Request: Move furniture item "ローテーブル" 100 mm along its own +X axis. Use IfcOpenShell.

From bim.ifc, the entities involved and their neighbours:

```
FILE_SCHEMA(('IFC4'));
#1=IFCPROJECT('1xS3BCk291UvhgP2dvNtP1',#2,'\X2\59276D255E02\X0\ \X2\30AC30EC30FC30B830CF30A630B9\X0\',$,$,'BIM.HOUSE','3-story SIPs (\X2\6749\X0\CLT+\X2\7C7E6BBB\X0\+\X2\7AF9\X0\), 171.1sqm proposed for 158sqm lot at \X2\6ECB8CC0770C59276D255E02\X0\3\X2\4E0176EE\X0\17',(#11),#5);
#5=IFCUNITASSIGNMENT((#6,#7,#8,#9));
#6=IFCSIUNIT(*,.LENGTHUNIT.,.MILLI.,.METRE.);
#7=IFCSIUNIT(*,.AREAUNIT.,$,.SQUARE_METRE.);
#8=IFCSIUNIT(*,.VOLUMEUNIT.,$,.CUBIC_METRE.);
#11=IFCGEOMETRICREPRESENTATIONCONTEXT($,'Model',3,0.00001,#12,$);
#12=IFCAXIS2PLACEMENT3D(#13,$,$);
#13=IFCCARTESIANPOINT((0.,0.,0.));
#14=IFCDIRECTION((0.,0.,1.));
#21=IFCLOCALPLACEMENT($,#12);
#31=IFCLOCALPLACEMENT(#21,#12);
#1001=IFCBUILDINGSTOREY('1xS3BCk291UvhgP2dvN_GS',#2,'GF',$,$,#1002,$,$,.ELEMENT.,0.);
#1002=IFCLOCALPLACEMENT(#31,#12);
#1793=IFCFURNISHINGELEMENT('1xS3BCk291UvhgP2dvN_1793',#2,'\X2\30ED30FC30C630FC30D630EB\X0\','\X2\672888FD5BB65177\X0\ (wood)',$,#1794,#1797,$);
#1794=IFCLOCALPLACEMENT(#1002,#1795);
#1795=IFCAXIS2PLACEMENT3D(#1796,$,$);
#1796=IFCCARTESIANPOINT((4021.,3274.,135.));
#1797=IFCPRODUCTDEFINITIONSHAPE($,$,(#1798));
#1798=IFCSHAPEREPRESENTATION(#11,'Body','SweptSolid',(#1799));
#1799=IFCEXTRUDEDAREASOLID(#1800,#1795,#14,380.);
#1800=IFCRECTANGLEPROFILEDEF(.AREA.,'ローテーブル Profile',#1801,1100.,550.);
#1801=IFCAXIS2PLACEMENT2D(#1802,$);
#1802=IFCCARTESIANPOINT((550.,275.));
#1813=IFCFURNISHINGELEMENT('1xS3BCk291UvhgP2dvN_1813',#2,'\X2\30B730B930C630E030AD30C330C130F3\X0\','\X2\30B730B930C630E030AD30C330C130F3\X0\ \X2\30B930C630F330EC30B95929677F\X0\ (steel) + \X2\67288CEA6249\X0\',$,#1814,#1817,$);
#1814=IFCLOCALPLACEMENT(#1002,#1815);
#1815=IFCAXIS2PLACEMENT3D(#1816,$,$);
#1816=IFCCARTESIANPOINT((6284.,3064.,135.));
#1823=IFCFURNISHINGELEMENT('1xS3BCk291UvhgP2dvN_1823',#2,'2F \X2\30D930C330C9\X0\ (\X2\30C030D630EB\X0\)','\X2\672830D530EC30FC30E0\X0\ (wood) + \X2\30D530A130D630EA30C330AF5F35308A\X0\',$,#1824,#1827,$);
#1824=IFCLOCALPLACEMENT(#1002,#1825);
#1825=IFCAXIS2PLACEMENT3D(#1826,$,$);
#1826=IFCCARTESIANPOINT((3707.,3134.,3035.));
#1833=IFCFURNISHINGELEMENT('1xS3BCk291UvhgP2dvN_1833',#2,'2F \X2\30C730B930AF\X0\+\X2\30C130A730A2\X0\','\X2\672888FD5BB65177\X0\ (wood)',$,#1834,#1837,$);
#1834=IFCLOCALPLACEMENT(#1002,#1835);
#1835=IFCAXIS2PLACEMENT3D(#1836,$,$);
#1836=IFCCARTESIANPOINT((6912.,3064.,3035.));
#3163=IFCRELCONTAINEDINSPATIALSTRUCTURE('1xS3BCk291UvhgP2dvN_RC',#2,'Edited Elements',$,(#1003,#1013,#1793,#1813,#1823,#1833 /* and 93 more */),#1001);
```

```python
import ifcopenshell
import ifcopenshell.api.geometry
import ifcopenshell.util.placement
import ifcopenshell.util.unit

model = ifcopenshell.open("bim.ifc")
unit_scale = ifcopenshell.util.unit.calculate_unit_scale(model)

item = model.by_guid("1xS3BCk291UvhgP2dvN_1793")
matrix = ifcopenshell.util.placement.get_local_placement(item.ObjectPlacement)
matrix[:3, 3] += matrix[:3, 0] * 0.1 / unit_scale
ifcopenshell.api.geometry.edit_object_placement(model, product=item, matrix=matrix, is_si=False)

print(ifcopenshell.util.placement.get_local_placement(item.ObjectPlacement).round(3) + 0.0)

model.write("bim-out.ifc")
```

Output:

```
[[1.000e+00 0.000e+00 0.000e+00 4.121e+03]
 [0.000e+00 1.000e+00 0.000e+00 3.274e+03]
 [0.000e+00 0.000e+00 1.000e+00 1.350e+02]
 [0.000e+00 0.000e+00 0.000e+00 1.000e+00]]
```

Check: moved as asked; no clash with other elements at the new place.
